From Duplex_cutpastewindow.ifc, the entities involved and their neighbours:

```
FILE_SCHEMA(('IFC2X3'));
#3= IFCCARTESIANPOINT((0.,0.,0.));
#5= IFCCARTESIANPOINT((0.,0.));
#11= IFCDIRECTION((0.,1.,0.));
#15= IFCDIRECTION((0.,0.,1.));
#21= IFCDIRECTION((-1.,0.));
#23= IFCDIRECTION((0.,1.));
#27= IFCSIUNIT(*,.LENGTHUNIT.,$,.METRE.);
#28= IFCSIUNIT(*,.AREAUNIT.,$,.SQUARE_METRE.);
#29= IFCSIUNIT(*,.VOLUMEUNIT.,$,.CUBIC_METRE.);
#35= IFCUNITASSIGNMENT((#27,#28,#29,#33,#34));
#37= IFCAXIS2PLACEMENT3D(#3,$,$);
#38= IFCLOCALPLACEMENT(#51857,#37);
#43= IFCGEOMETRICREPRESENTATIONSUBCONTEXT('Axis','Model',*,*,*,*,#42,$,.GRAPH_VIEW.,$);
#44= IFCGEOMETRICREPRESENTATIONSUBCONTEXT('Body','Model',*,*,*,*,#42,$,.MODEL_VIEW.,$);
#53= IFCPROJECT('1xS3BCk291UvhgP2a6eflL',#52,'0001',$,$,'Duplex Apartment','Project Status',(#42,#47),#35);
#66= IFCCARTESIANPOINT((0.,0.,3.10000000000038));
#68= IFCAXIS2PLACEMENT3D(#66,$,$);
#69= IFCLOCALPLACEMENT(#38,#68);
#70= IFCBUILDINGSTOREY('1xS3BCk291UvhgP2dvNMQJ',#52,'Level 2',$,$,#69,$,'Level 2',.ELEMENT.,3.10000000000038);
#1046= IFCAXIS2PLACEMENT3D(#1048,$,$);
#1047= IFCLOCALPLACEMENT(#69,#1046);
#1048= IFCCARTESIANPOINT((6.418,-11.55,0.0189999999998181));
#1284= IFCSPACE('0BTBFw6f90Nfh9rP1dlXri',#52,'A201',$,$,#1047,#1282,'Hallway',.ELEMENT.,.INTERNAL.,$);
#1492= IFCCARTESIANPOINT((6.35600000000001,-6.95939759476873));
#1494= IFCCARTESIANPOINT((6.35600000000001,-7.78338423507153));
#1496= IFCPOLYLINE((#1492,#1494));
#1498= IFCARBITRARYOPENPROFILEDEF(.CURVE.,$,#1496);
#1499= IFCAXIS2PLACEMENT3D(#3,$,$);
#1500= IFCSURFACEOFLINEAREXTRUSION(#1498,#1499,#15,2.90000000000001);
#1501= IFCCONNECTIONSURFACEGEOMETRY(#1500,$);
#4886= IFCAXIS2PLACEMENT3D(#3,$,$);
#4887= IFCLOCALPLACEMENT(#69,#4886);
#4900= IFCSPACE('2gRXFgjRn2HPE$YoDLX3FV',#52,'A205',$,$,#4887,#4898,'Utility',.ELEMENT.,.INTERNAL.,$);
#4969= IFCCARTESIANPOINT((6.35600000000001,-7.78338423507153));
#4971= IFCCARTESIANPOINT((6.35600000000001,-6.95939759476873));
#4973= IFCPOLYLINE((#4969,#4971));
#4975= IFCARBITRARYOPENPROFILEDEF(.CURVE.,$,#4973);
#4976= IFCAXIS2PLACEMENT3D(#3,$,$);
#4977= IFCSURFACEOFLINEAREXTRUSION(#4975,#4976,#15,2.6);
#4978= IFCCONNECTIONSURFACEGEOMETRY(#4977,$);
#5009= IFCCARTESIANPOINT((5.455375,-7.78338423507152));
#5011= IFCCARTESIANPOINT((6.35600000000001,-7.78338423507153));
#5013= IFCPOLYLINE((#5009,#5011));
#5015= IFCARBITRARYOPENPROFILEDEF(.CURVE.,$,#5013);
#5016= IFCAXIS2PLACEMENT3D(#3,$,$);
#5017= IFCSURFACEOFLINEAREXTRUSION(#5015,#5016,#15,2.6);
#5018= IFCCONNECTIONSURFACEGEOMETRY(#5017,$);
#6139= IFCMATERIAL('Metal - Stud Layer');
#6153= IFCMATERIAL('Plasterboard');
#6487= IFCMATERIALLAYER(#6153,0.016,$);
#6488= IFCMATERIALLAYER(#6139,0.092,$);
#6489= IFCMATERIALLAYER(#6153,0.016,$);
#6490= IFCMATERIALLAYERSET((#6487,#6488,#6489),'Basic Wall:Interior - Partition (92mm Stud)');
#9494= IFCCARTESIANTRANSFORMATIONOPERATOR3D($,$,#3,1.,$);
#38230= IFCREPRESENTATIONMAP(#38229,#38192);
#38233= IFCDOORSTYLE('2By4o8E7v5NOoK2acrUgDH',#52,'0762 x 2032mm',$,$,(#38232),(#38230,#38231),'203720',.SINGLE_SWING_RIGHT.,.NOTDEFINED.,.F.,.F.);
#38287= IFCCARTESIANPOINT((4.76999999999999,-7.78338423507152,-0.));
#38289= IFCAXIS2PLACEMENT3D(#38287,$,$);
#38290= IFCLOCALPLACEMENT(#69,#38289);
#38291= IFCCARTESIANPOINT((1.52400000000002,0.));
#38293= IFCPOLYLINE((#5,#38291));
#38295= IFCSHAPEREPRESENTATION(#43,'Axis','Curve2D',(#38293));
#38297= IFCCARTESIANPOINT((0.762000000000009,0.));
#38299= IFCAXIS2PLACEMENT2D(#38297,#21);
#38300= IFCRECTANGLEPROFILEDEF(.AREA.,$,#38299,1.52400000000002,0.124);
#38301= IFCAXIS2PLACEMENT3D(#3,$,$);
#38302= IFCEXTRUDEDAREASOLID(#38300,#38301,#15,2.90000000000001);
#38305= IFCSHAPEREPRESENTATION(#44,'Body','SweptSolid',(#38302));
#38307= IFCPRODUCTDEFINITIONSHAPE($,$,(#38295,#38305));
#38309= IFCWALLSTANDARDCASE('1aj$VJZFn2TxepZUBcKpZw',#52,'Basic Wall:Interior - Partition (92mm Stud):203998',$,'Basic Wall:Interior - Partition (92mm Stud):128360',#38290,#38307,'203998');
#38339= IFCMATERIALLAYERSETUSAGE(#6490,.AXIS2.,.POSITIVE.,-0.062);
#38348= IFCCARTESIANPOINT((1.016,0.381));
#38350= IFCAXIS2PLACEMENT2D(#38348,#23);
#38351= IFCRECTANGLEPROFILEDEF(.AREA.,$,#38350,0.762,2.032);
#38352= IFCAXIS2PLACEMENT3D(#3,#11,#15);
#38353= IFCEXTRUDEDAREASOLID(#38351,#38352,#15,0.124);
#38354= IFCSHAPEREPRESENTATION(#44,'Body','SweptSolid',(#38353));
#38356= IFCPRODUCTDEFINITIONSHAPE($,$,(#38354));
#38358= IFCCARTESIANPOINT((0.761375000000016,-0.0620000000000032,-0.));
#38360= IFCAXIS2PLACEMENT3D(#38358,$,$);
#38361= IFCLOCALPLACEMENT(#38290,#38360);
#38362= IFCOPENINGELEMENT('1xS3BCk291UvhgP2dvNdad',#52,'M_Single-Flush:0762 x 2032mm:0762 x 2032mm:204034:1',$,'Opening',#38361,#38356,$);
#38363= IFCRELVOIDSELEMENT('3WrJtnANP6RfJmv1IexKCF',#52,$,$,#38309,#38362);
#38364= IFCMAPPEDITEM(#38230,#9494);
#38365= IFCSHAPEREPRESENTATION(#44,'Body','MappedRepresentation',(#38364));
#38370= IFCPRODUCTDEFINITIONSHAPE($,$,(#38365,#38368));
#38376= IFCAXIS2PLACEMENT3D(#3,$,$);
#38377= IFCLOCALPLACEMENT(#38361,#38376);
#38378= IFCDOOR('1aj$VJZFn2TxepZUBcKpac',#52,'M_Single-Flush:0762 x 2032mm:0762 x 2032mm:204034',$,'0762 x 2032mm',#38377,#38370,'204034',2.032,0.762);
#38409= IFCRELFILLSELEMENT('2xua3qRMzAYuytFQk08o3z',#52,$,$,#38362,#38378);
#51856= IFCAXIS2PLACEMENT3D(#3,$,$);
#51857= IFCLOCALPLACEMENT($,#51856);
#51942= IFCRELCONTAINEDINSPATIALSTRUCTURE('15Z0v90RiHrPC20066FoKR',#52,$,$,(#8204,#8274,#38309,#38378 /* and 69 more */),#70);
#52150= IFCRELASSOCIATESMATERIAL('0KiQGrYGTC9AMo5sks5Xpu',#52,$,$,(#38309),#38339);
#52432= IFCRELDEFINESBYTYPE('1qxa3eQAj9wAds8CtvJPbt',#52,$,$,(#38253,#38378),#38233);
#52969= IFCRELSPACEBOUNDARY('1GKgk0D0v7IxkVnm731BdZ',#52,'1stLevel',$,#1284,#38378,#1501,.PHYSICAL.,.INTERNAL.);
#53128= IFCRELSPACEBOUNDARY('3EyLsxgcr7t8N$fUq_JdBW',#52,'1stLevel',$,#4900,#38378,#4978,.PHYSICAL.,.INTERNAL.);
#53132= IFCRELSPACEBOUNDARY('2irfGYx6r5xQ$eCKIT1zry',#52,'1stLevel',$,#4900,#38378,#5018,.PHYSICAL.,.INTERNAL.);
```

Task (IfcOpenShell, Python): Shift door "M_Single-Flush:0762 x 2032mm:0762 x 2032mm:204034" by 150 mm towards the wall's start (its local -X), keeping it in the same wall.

```python
import numpy as np
import ifcopenshell
import ifcopenshell.api.geometry
import ifcopenshell.util.placement

model = ifcopenshell.open("Duplex_cutpastewindow.ifc")

door = model.by_guid("1aj$VJZFn2TxepZUBcKpac")
opening = door.FillsVoids[0].RelatingOpeningElement
wall = opening.VoidsElements[0].RelatingBuildingElement

wall_matrix = ifcopenshell.util.placement.get_local_placement(wall.ObjectPlacement)
shift = wall_matrix[:3, 0] * -0.15
before = ifcopenshell.util.placement.get_local_placement(door.ObjectPlacement)[:3, 3].copy()

# The door is placed relative to its opening, so it follows when the opening moves.
matrix = ifcopenshell.util.placement.get_local_placement(opening.ObjectPlacement)
matrix[:3, 3] += shift
ifcopenshell.api.geometry.edit_object_placement(
    model, product=opening, matrix=matrix, is_si=False, should_transform_children=True
)

# Space boundary surfaces are stored in each space's coordinates; move them too.
for rel in door.ProvidesBoundaries:
    if not rel.ConnectionGeometry:
        continue
    surface = rel.ConnectionGeometry.SurfaceOnRelatingElement
    space_matrix = ifcopenshell.util.placement.get_local_placement(rel.RelatingSpace.ObjectPlacement)
    point = np.array(surface.Position.Location.Coordinates) + space_matrix[:3, :3].T @ shift
    surface.Position = model.createIfcAxis2Placement3D(
        model.createIfcCartesianPoint(point.tolist()), surface.Position.Axis, surface.Position.RefDirection
    )

after = ifcopenshell.util.placement.get_local_placement(door.ObjectPlacement)[:3, 3]
print("door moved by", (after - before).round(3) + 0.0)

model.write("Duplex_cutpastewindow-out.ifc")
```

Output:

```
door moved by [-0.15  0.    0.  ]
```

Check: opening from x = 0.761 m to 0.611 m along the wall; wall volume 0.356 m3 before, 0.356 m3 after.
